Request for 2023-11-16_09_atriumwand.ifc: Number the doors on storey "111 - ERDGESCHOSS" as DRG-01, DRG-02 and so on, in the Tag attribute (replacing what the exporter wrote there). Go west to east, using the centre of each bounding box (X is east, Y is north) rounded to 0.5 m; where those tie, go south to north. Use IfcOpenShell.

First a look at what the model holds.

```python
import ifcopenshell
import ifcopenshell.util.element
import ifcopenshell.util.placement

model = ifcopenshell.open("2023-11-16_09_atriumwand.ifc")
print(model.schema)
storey = next(s for s in model.by_type("IfcBuildingStorey") if s.Name == "111 - ERDGESCHOSS")
doors = [e for e in ifcopenshell.util.element.get_decomposition(storey) if e.is_a("IfcDoor")]
for e in sorted(doors, key=lambda e: e.id()):
    origin = ifcopenshell.util.placement.get_local_placement(e.ObjectPlacement)[:3, 3]
    print(e.id(), e.Tag, e.Name, origin.round(2) + 0.0, sep=" | ")
```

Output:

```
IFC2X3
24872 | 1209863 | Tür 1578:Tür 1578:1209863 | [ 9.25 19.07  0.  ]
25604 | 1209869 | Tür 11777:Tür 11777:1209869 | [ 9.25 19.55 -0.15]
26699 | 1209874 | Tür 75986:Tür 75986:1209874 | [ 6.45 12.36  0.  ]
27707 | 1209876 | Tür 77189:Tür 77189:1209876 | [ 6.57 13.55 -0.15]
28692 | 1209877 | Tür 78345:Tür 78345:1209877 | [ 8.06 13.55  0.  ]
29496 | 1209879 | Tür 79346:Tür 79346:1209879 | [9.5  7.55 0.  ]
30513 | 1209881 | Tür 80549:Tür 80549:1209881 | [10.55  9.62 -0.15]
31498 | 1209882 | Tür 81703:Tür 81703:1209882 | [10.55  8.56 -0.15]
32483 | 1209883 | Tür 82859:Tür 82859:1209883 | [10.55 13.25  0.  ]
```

```python
import ifcopenshell
import ifcopenshell.geom
import ifcopenshell.util.element
import ifcopenshell.util.shape

model = ifcopenshell.open("2023-11-16_09_atriumwand.ifc")
settings = ifcopenshell.geom.settings()
settings.set("use-world-coords", True)


def centre(element):
    shape = ifcopenshell.geom.create_shape(settings, element)
    return ifcopenshell.util.shape.get_bbox_centroid(shape.geometry)


storey = next(s for s in model.by_type("IfcBuildingStorey") if s.Name == "111 - ERDGESCHOSS")
doors = [e for e in ifcopenshell.util.element.get_decomposition(storey) if e.is_a("IfcDoor")]

# Insertion points can sit at a corner or the storey origin, so sort by the geometry (in metres).
centres = {e: centre(e) for e in doors}
doors.sort(key=lambda e: (round(centres[e][0] / 0.5), centres[e][1]))

for i, e in enumerate(doors, start=1):
    number = f"DRG-{i:02d}"
    e.Tag = number
    print(e.id(), number)

model.write("2023-11-16_09_atriumwand_rev.ifc")
```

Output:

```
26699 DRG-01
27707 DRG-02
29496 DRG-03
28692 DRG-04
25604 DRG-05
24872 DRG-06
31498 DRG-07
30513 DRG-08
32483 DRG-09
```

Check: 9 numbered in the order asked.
